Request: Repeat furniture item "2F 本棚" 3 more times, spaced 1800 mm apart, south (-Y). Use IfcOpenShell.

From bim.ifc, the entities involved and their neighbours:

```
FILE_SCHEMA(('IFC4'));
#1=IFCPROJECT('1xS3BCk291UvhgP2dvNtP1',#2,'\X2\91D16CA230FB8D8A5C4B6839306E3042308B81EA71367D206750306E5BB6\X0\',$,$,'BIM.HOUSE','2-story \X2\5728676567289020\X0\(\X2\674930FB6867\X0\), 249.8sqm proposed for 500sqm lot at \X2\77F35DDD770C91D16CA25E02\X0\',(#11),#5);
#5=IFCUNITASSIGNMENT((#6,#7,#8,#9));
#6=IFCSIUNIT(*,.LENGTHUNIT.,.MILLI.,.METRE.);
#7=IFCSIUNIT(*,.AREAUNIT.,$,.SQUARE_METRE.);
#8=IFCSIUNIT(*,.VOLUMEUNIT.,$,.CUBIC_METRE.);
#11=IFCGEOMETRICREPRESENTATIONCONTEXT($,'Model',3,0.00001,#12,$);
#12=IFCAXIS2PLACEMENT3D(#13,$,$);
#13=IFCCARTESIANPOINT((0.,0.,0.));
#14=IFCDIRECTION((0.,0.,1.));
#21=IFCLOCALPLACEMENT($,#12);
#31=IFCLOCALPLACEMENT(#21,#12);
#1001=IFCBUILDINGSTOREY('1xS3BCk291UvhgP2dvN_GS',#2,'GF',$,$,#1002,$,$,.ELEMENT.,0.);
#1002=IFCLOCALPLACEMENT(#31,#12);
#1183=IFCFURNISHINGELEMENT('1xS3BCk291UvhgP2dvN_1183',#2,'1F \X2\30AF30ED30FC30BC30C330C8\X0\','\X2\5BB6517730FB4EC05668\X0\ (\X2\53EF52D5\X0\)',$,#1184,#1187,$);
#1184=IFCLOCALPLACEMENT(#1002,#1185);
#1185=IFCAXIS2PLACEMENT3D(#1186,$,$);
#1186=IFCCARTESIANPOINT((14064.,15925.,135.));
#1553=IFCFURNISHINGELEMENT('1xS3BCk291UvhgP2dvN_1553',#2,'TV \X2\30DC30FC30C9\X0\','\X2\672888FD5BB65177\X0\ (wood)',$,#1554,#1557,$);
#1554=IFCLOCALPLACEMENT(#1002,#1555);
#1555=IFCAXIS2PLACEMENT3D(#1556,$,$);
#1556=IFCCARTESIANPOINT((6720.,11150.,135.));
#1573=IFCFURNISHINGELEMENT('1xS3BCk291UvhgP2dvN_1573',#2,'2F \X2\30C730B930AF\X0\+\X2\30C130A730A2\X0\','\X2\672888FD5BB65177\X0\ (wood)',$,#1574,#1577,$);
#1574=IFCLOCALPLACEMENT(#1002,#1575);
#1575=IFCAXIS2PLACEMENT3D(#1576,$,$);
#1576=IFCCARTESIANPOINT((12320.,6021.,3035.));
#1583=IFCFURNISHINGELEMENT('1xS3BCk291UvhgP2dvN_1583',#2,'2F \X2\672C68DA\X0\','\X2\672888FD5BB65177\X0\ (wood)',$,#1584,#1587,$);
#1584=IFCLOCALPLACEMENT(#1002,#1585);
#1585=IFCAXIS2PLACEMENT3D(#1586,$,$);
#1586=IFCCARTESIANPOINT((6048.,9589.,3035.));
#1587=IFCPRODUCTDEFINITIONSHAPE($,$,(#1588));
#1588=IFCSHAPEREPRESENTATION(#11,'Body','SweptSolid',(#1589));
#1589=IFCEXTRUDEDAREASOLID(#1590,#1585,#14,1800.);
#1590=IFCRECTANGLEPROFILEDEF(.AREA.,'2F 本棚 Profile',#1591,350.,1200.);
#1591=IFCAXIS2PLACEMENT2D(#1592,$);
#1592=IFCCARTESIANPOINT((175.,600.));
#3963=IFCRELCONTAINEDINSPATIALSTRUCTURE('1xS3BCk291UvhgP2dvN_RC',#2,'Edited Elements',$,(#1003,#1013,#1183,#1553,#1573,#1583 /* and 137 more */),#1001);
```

```python
import numpy as np
import ifcopenshell
import ifcopenshell.api.geometry
import ifcopenshell.api.root
import ifcopenshell.util.element
import ifcopenshell.util.placement
import ifcopenshell.util.unit

model = ifcopenshell.open("bim.ifc")
unit_scale = ifcopenshell.util.unit.calculate_unit_scale(model)


def reuse_history(source, copy):
    """copy_class also copies each property set's owner history, people and application; keep the originals."""
    for rel in copy.IsDefinedBy:
        if rel.is_a("IfcRelDefinesByProperties") and (history := rel.RelatingPropertyDefinition.OwnerHistory):
            rel.RelatingPropertyDefinition.OwnerHistory = source.OwnerHistory
            ifcopenshell.util.element.remove_deep2(model, history)


source = model.by_id(1583)
base = ifcopenshell.util.placement.get_local_placement(source.ObjectPlacement)
step = np.array([0.0, -1.0, 0.0]) * 1.8 / unit_scale

for i in range(1, 4):
    copy = ifcopenshell.api.root.copy_class(model, product=source)
    copy.Representation = ifcopenshell.util.element.copy_deep(
        model, source.Representation, exclude=["IfcGeometricRepresentationContext", "IfcRepresentationMap"]
    )
    reuse_history(source, copy)
    matrix = base.copy()
    matrix[:3, 3] += i * step
    print("added at", matrix[:3, 3].round(3) + 0.0)
    ifcopenshell.api.geometry.edit_object_placement(model, product=copy, matrix=matrix, is_si=False)

model.write("bim_rev.ifc")
```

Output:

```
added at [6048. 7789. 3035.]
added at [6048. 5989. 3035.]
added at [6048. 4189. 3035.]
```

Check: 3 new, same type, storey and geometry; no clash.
